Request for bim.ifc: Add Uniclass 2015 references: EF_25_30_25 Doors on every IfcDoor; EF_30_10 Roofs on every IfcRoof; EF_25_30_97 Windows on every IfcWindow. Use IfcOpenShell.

First a look at what the model holds.

```python
import ifcopenshell

model = ifcopenshell.open("bim.ifc")
print(model.schema)
print("classifications:", [c.Name for c in model.by_type("IfcClassification")])
for ifc_class in ("IfcDoor", "IfcRoof", "IfcStair", "IfcWall", "IfcWindow"):
    print(ifc_class, len(model.by_type(ifc_class)))
```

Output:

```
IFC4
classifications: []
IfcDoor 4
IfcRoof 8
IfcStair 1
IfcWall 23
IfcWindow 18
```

```python
import ifcopenshell
import ifcopenshell.api.classification

model = ifcopenshell.open("bim.ifc")

system = ifcopenshell.api.classification.add_classification(model, classification="Uniclass 2015")

codes = {
    "IfcDoor": ("EF_25_30_25", "Doors"),
    "IfcRoof": ("EF_30_10", "Roofs"),
    "IfcWindow": ("EF_25_30_97", "Windows"),
}
for ifc_class, (code, name) in codes.items():
    products = model.by_type(ifc_class)
    ifcopenshell.api.classification.add_reference(
        model, products=products, classification=system, identification=code, name=name
    )
    print(code, len(products))

model.write("bim_rev.ifc")
```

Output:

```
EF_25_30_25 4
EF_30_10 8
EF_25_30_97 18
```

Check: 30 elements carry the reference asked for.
